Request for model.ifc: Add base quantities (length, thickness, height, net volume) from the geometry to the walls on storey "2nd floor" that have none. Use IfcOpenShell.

First a look at what the model holds.

```python
import ifcopenshell
import ifcopenshell.util.element
import ifcopenshell.util.unit

model = ifcopenshell.open("model.ifc")
print(model.schema)
for unit_type in ("LENGTHUNIT", "AREAUNIT", "VOLUMEUNIT"):
    print(unit_type, ifcopenshell.util.unit.calculate_unit_scale(model, unit_type))
storey = next(s for s in model.by_type("IfcBuildingStorey") if s.Name == "2nd floor")
walls = [e for e in ifcopenshell.util.element.get_decomposition(storey) if e.is_a("IfcWall")]
for e in sorted(walls, key=lambda e: e.id()):
    print(e.id(), e.is_a(), e.Name, list(ifcopenshell.util.element.get_psets(e, qtos_only=True)), sep=" | ")
```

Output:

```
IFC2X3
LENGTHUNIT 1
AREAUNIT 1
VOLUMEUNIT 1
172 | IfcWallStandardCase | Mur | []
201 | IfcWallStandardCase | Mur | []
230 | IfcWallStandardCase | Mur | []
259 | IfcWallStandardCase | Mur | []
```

```python
import ifcopenshell
import ifcopenshell.api.pset
import ifcopenshell.geom
import ifcopenshell.util.element
import ifcopenshell.util.shape
import ifcopenshell.util.unit

model = ifcopenshell.open("model.ifc")
unit_scale = ifcopenshell.util.unit.calculate_unit_scale(model)
volume_scale = ifcopenshell.util.unit.calculate_unit_scale(model, "VOLUMEUNIT")
settings = ifcopenshell.geom.settings()

storey = next(s for s in model.by_type("IfcBuildingStorey") if s.Name == "2nd floor")
walls = [e for e in ifcopenshell.util.element.get_decomposition(storey) if e.is_a("IfcWall")]

for e in sorted(walls, key=lambda e: e.id()):
    if ifcopenshell.util.element.get_psets(e, qtos_only=True, should_inherit=False):
        continue
    # Geometry comes back in metres, in the element's own axes.
    shape = ifcopenshell.geom.create_shape(settings, e)
    values = {
        "Length": ifcopenshell.util.shape.get_x(shape.geometry) / unit_scale,
        "Width": ifcopenshell.util.shape.get_y(shape.geometry) / unit_scale,
        "Height": ifcopenshell.util.shape.get_z(shape.geometry) / unit_scale,
        "NetVolume": ifcopenshell.util.shape.get_volume(shape.geometry) / volume_scale,
    }
    qto = ifcopenshell.api.pset.add_qto(model, product=e, name="BaseQuantities")
    ifcopenshell.api.pset.edit_qto(model, qto=qto, properties=values)
    print(e.id(), {k: round(v, 3) for k, v in values.items()})

model.write("model_edited.ifc")
```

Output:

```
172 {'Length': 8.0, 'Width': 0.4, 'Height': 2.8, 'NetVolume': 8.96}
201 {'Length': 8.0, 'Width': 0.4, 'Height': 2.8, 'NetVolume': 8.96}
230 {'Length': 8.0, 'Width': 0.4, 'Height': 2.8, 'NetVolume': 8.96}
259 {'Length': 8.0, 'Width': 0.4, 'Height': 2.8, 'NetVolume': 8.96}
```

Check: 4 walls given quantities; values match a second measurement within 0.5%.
